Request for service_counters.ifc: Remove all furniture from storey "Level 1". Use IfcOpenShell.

First a look at what the model holds.

```python
import ifcopenshell
import ifcopenshell.util.element

model = ifcopenshell.open("service_counters.ifc")
print(model.schema)
storey = next(s for s in model.by_type("IfcBuildingStorey") if s.Name == "Level 1")
furniture = [e for e in ifcopenshell.util.element.get_decomposition(storey) if e.is_a("IfcFurnishingElement")]
seen = {}
for e in furniture:
    element_type = ifcopenshell.util.element.get_type(e)
    name = element_type.Name if element_type not in (None, e) else None
    seen[name] = seen.get(name, 0) + 1
for name, count in sorted(seen.items(), key=str):
    print(count, "x", name)
```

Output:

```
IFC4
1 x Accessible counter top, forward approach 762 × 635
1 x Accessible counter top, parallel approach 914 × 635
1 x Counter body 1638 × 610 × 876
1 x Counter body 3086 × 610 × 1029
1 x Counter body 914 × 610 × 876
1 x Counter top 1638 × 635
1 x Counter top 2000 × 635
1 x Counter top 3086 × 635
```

```python
import ifcopenshell
import ifcopenshell.api.root
import ifcopenshell.util.element

model = ifcopenshell.open("service_counters.ifc")

storey = next(s for s in model.by_type("IfcBuildingStorey") if s.Name == "Level 1")
furniture = [e for e in ifcopenshell.util.element.get_decomposition(storey) if e.is_a("IfcFurnishingElement")]

for e in furniture:
    ifcopenshell.api.root.remove_product(model, product=e)
print(len(furniture), "removed")

model.write("service_counters_updated.ifc")
```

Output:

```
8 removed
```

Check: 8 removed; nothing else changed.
